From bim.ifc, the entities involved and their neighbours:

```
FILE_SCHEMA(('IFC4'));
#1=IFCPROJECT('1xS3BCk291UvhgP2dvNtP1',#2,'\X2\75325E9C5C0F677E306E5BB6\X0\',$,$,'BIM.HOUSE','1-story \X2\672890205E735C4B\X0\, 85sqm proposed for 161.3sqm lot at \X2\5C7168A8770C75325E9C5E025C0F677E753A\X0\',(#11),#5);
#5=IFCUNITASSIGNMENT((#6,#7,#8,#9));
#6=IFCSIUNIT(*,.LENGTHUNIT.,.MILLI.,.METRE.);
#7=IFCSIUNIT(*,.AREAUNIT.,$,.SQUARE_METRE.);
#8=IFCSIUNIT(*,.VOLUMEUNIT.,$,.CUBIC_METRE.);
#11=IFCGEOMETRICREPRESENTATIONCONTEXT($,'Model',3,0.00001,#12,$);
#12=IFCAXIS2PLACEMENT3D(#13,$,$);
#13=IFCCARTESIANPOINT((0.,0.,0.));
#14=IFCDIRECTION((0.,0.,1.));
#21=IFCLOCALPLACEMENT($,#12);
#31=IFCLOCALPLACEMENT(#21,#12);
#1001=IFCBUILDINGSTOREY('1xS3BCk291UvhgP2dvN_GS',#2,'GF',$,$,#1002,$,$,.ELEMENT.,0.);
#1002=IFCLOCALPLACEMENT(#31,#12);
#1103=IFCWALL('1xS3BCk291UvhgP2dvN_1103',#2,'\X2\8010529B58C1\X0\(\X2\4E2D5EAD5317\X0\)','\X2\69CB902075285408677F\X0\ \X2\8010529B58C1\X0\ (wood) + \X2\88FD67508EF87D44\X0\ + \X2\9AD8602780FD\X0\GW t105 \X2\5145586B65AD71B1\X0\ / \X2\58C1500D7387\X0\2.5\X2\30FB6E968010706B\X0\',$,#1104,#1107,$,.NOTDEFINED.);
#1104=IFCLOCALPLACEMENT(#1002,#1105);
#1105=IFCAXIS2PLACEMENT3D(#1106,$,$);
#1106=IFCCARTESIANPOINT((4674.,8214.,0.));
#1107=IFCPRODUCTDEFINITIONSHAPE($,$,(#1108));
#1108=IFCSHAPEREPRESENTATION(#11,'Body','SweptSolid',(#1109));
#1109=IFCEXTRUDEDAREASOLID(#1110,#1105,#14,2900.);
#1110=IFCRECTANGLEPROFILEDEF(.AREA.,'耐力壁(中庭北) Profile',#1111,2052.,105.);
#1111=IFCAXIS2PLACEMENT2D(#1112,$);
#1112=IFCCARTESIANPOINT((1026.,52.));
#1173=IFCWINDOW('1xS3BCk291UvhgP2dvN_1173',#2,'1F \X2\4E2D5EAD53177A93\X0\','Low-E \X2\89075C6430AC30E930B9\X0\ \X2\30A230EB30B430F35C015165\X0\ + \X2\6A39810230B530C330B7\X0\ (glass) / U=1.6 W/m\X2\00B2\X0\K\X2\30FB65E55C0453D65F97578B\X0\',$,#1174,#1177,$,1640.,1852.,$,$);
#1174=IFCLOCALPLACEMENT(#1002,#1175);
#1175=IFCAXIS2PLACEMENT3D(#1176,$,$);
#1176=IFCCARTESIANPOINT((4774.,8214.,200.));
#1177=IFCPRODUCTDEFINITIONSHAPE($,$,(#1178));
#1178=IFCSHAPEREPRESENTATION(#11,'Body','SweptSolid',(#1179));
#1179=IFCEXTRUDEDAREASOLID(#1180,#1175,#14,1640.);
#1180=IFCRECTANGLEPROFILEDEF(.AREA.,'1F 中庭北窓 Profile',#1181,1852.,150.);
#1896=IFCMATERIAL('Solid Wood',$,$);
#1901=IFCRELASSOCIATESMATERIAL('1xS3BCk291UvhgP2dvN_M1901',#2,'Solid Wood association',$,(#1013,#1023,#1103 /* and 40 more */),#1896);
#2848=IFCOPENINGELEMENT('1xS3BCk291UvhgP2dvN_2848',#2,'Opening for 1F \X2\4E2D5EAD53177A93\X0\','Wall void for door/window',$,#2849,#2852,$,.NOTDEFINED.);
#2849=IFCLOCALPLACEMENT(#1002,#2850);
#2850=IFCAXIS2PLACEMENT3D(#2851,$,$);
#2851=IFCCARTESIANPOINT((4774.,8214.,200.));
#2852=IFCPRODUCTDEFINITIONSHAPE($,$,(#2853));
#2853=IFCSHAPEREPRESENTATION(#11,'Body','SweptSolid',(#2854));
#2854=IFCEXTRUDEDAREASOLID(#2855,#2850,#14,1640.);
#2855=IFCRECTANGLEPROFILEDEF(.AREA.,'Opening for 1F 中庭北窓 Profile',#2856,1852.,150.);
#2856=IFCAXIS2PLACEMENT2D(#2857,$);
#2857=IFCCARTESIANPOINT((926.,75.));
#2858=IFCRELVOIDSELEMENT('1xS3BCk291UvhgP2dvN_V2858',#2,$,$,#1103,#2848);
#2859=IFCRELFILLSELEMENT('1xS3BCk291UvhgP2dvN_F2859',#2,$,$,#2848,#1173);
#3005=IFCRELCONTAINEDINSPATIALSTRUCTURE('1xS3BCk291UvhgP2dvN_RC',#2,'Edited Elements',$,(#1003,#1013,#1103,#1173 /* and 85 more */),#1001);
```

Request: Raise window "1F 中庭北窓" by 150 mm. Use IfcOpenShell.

```python
import numpy as np
import ifcopenshell
import ifcopenshell.api.geometry
import ifcopenshell.util.placement
import ifcopenshell.util.unit

model = ifcopenshell.open("bim.ifc")
unit_scale = ifcopenshell.util.unit.calculate_unit_scale(model)

window = model.by_id(1173)
opening = window.FillsVoids[0].RelatingOpeningElement
dz = 150.0

shift = np.array([0.0, 0.0, dz])
# The window is not placed relative to its opening, so move both.
for product in (opening, window):
    matrix = ifcopenshell.util.placement.get_local_placement(product.ObjectPlacement)
    matrix[:3, 3] += shift
    ifcopenshell.api.geometry.edit_object_placement(model, product=product, matrix=matrix, is_si=False)

print(f"moved by {dz * unit_scale:+.3f} m")

model.write("bim_updated.ifc")
```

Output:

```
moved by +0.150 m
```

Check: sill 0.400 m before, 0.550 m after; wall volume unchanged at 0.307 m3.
